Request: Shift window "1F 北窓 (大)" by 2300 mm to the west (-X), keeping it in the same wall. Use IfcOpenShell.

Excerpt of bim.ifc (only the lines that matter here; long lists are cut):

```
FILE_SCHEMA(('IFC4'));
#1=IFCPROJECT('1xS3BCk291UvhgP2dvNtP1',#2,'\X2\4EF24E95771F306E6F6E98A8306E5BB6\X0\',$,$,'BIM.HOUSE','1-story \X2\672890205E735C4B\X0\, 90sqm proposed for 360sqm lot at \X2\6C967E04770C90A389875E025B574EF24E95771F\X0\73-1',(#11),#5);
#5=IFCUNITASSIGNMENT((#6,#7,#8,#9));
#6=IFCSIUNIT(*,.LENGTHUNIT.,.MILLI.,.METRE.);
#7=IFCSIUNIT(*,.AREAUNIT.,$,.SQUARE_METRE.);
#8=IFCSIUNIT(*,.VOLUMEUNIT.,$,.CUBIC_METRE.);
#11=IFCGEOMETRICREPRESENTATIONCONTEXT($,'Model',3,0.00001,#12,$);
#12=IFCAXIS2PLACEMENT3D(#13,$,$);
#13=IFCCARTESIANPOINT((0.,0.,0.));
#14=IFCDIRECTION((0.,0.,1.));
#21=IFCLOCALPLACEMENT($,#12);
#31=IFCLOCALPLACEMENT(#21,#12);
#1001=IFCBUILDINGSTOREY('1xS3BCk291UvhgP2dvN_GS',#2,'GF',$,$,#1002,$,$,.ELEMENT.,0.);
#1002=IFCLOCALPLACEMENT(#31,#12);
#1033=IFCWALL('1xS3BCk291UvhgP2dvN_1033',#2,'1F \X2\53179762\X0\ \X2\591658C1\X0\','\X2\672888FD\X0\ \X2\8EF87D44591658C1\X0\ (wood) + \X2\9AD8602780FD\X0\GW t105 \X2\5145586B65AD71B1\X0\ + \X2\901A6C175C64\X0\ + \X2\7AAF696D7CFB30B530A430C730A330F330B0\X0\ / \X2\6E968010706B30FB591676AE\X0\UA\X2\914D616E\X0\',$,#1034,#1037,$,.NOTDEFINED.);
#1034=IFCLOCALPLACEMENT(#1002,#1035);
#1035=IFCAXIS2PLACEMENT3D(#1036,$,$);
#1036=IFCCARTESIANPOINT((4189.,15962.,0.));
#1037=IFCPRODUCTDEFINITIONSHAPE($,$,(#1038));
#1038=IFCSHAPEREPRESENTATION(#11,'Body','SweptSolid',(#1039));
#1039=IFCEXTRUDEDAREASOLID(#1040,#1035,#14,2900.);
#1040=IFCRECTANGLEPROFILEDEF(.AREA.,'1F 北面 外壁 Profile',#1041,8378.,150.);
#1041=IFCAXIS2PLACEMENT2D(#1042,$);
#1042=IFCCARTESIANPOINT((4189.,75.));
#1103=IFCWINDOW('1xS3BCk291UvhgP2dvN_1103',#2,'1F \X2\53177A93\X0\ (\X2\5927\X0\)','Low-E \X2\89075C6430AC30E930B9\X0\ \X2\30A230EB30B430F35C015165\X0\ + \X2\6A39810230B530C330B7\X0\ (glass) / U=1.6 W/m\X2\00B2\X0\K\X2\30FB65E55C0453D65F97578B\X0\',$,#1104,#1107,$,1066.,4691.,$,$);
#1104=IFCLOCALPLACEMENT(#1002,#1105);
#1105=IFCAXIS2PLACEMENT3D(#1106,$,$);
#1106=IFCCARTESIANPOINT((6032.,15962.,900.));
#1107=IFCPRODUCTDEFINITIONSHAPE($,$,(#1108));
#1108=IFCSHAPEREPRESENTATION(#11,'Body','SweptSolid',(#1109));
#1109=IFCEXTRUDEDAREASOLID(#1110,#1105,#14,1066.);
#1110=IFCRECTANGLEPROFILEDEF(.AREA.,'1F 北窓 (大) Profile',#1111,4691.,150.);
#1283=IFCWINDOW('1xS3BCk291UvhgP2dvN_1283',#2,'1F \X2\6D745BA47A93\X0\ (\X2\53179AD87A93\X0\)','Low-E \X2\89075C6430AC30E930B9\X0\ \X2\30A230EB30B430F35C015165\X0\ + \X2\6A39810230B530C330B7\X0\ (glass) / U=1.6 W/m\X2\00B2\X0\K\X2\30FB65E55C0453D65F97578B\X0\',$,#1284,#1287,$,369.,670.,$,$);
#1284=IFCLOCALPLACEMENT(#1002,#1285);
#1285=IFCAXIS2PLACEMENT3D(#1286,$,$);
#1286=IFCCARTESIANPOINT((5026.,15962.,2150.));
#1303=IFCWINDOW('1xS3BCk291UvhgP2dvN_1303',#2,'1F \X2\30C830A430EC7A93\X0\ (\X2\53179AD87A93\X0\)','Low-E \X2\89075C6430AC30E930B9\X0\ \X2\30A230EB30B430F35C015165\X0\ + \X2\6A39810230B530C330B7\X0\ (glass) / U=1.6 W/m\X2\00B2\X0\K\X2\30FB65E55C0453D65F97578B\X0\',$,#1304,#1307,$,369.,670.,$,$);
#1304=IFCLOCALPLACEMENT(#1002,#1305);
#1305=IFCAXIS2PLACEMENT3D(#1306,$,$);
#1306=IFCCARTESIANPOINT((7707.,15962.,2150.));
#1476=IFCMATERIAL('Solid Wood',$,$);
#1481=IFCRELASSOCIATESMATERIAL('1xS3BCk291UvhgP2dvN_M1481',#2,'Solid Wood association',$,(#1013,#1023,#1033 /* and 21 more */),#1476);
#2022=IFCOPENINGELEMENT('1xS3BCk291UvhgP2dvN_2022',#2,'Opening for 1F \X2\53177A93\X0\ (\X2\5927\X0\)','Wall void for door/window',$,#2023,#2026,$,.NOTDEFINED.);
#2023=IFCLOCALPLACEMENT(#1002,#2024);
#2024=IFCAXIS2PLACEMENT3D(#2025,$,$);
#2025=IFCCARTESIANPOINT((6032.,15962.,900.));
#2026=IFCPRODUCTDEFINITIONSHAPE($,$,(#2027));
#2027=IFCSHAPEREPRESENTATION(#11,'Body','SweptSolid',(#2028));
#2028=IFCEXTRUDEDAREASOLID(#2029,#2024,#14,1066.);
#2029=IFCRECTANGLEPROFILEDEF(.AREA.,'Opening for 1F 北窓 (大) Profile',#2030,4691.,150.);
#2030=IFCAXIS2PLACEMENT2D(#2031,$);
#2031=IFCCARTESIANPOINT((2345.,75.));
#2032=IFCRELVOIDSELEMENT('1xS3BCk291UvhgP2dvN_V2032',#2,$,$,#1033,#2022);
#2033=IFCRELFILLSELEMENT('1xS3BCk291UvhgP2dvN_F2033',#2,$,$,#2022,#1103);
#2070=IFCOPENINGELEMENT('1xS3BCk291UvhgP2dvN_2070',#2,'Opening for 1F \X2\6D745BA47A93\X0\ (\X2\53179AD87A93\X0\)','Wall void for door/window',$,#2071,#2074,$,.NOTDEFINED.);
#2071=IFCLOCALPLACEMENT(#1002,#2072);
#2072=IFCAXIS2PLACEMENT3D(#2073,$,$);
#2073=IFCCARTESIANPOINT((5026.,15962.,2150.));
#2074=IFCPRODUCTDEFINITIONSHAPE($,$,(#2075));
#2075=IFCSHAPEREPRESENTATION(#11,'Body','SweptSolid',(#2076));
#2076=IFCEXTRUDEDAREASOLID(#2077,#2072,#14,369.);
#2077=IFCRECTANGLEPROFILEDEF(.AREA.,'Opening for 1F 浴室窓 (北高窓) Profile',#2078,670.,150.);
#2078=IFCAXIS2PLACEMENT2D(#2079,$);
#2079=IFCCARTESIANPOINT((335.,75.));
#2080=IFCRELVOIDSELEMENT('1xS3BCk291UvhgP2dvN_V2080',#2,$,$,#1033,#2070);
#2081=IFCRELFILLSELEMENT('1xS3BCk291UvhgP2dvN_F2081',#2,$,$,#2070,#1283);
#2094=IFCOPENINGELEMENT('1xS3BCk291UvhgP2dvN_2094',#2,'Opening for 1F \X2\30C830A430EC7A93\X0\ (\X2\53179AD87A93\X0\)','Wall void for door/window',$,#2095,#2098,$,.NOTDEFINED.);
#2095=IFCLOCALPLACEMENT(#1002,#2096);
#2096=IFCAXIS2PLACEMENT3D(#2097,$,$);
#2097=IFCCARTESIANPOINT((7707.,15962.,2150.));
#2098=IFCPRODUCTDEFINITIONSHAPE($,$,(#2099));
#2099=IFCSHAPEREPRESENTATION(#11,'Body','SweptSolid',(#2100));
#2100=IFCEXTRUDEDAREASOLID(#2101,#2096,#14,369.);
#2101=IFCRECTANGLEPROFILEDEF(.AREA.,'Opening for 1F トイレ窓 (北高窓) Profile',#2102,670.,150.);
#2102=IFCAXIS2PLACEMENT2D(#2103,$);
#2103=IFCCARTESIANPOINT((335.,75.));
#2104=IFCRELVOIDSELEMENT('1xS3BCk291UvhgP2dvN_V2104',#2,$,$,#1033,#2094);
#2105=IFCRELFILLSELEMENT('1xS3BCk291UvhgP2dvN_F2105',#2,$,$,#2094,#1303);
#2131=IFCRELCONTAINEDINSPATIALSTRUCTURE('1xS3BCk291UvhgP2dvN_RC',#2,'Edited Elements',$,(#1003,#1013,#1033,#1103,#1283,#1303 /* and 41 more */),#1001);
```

```python
import ifcopenshell
import ifcopenshell.api.geometry
import ifcopenshell.util.placement
import ifcopenshell.util.unit

model = ifcopenshell.open("bim.ifc")
unit_scale = ifcopenshell.util.unit.calculate_unit_scale(model)

window = model.by_guid("1xS3BCk291UvhgP2dvN_1103")
opening = window.FillsVoids[0].RelatingOpeningElement
wall = opening.VoidsElements[0].RelatingBuildingElement

wall_matrix = ifcopenshell.util.placement.get_local_placement(wall.ObjectPlacement)
shift = wall_matrix[:3, 0] * -2.3 / unit_scale
before = ifcopenshell.util.placement.get_local_placement(window.ObjectPlacement)[:3, 3].copy()

# The window is not placed relative to its opening, so move both.
for product in (opening, window):
    matrix = ifcopenshell.util.placement.get_local_placement(product.ObjectPlacement)
    matrix[:3, 3] += shift
    ifcopenshell.api.geometry.edit_object_placement(model, product=product, matrix=matrix, is_si=False)

after = ifcopenshell.util.placement.get_local_placement(window.ObjectPlacement)[:3, 3]
print("window moved by", (after - before).round(3) + 0.0)

model.write("bim_edited.ifc")
```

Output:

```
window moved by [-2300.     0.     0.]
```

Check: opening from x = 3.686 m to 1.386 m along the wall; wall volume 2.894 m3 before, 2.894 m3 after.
